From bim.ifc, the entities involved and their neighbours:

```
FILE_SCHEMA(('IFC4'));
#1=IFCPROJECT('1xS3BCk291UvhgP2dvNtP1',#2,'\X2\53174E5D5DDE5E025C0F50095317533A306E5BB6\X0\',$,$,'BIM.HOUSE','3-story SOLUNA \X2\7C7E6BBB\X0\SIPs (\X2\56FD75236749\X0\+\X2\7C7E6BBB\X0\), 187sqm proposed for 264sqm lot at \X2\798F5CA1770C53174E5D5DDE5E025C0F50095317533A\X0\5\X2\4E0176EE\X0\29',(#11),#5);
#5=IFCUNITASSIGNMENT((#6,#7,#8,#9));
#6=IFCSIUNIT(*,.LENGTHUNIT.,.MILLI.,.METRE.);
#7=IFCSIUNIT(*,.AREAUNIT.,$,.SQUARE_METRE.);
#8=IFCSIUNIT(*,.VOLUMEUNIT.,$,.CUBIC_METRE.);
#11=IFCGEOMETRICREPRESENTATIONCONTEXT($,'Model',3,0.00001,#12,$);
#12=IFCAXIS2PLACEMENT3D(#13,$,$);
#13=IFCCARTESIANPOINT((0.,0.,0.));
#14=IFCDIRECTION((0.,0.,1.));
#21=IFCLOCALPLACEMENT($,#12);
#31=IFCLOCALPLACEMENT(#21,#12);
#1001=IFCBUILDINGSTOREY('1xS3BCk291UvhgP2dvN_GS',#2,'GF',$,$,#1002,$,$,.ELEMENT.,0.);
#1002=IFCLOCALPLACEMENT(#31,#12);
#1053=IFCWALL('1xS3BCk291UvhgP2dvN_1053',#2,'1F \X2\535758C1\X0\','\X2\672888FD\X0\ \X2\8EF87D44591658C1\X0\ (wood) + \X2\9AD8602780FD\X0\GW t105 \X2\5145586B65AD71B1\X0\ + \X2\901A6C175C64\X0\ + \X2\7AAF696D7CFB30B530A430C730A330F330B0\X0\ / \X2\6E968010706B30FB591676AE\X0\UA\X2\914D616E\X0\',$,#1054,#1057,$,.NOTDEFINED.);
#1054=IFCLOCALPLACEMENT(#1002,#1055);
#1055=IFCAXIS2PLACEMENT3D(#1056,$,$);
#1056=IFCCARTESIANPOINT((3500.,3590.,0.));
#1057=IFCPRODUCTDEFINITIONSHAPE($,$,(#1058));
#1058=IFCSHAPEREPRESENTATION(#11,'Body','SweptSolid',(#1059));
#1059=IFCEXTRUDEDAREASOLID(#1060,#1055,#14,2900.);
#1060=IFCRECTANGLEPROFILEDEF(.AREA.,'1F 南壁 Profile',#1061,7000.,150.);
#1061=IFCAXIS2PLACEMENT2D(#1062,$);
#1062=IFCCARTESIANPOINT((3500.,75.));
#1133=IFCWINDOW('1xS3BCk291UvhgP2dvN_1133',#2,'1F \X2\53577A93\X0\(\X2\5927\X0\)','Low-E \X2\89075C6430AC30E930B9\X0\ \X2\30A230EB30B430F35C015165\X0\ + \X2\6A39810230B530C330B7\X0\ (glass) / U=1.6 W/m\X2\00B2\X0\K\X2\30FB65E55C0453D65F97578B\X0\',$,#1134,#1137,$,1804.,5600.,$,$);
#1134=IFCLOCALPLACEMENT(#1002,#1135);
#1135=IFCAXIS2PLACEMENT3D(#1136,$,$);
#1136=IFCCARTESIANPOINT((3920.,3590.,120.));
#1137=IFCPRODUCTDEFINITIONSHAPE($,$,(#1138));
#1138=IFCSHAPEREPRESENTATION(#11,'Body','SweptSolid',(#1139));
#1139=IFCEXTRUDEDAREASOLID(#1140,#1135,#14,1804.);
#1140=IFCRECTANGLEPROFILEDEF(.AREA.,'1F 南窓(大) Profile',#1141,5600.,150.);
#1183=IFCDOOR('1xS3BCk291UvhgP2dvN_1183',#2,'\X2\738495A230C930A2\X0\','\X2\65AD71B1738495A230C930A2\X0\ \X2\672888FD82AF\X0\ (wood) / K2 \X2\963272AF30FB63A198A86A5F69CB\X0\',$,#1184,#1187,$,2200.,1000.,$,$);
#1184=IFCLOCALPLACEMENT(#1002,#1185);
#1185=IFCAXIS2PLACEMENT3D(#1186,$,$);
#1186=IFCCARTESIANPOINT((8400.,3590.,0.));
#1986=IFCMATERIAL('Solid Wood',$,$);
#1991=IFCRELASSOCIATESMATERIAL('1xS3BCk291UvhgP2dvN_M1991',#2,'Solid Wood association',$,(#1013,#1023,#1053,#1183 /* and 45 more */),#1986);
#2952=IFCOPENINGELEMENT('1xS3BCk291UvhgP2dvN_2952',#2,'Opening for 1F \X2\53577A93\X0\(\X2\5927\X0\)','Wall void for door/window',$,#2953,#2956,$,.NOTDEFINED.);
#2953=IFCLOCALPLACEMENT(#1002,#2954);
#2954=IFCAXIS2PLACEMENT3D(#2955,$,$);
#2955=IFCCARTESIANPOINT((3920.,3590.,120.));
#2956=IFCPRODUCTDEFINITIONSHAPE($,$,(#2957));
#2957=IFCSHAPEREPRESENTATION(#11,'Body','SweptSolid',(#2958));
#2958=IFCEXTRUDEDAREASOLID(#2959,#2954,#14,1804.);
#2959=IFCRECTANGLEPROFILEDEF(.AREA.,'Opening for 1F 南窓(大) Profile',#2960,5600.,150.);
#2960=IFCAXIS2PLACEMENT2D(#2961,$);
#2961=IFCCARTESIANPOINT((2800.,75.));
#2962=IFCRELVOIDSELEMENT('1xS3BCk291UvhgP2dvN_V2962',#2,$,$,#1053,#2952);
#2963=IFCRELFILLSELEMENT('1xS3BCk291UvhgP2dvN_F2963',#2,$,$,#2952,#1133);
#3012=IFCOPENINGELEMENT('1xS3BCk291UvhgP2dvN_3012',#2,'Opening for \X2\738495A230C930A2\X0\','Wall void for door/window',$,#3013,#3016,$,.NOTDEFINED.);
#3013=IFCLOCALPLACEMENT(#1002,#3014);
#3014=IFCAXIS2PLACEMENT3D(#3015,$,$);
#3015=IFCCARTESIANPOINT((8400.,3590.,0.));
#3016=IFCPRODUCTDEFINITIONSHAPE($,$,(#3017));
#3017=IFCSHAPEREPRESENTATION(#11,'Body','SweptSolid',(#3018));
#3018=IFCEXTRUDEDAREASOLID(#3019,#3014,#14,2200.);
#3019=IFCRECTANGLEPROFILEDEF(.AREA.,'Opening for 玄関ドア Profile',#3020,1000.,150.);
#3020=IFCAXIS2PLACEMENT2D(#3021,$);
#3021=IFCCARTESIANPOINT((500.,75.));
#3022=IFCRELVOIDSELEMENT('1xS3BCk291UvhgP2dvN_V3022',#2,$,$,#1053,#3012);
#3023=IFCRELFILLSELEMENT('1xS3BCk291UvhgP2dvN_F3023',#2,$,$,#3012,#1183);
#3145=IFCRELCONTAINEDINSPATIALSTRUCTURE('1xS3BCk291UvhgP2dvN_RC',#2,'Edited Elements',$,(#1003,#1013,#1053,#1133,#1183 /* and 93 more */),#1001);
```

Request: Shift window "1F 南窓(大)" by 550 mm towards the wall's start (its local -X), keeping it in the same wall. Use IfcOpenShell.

```python
import ifcopenshell
import ifcopenshell.api.geometry
import ifcopenshell.util.placement

model = ifcopenshell.open("bim.ifc")

window = model.by_guid("1xS3BCk291UvhgP2dvN_1133")
opening = window.FillsVoids[0].RelatingOpeningElement
wall = opening.VoidsElements[0].RelatingBuildingElement

wall_matrix = ifcopenshell.util.placement.get_local_placement(wall.ObjectPlacement)
shift = wall_matrix[:3, 0] * -550.0
before = ifcopenshell.util.placement.get_local_placement(window.ObjectPlacement)[:3, 3].copy()

# The window is not placed relative to its opening, so move both.
for product in (opening, window):
    matrix = ifcopenshell.util.placement.get_local_placement(product.ObjectPlacement)
    matrix[:3, 3] += shift
    ifcopenshell.api.geometry.edit_object_placement(model, product=product, matrix=matrix, is_si=False)

after = ifcopenshell.util.placement.get_local_placement(window.ObjectPlacement)[:3, 3]
print("window moved by", (after - before).round(3) + 0.0)

model.write("bim_v2.ifc")
```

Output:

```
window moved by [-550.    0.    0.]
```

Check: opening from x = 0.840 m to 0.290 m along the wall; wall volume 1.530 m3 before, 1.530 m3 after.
